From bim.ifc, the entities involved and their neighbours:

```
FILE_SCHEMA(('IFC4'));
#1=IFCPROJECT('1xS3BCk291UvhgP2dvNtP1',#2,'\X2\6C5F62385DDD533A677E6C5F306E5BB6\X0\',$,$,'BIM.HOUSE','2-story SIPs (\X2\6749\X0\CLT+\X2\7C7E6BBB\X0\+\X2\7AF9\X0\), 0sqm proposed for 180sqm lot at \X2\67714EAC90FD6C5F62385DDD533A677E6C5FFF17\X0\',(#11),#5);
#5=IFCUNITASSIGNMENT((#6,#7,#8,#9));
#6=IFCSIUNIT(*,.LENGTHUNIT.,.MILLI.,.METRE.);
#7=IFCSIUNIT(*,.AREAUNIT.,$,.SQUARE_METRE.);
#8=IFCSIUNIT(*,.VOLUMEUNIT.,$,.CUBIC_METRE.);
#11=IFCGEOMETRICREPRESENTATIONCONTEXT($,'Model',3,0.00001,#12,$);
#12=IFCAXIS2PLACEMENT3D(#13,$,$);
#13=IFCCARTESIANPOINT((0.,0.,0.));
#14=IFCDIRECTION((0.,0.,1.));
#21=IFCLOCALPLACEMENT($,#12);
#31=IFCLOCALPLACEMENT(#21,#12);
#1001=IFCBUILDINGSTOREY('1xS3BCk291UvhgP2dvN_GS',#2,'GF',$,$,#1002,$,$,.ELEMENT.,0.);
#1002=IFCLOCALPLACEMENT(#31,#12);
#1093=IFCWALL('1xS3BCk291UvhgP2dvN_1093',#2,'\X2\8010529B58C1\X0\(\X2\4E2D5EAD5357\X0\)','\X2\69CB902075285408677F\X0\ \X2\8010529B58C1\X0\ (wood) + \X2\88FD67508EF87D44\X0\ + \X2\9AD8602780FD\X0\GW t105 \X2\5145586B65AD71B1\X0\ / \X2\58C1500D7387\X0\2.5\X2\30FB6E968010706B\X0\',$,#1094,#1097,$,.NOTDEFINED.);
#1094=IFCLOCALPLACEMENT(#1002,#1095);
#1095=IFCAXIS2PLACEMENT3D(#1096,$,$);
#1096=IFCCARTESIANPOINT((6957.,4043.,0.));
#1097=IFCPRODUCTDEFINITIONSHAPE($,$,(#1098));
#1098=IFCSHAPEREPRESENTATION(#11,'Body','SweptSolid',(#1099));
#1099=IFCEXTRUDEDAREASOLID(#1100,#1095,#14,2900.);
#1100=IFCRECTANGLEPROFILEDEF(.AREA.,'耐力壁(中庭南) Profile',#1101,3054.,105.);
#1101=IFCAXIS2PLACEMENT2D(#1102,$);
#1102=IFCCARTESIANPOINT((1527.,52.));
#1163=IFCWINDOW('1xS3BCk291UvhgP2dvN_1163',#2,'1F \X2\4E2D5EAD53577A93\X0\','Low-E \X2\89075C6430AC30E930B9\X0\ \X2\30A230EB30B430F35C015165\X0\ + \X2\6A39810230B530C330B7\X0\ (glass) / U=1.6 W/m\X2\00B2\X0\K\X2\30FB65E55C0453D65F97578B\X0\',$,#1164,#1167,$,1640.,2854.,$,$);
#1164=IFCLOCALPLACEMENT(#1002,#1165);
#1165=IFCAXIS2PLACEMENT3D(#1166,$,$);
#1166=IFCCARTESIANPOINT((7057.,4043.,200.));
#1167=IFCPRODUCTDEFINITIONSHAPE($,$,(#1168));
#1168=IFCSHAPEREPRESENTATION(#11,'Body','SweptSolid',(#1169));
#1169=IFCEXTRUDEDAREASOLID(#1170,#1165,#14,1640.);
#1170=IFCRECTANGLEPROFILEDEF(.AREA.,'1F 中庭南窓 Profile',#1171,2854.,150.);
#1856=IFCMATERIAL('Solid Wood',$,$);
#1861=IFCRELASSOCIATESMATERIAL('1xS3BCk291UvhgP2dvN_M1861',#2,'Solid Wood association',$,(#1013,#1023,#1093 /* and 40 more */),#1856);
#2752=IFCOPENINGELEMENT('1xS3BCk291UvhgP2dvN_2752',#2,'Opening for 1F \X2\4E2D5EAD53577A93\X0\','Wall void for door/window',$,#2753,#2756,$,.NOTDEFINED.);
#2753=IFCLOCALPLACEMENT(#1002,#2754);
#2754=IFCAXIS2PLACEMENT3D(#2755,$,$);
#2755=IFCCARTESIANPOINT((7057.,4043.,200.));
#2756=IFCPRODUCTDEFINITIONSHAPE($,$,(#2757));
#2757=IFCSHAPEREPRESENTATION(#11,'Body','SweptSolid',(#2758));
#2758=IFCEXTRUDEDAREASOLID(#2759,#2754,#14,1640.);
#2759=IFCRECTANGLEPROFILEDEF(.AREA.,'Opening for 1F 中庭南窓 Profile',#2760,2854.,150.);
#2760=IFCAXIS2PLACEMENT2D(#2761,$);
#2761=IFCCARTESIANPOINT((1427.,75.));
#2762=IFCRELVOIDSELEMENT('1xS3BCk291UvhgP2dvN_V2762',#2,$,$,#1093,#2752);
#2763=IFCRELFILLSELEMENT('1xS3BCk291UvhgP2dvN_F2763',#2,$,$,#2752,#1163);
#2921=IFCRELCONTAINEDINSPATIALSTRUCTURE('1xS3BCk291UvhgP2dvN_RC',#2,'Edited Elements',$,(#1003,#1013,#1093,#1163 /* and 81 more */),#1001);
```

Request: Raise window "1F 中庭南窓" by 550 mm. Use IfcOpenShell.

```python
import numpy as np
import ifcopenshell
import ifcopenshell.api.geometry
import ifcopenshell.util.placement
import ifcopenshell.util.unit

model = ifcopenshell.open("bim.ifc")
unit_scale = ifcopenshell.util.unit.calculate_unit_scale(model)

window = model.by_guid("1xS3BCk291UvhgP2dvN_1163")
opening = window.FillsVoids[0].RelatingOpeningElement
dz = 0.55 / unit_scale

shift = np.array([0.0, 0.0, dz])
# The window is not placed relative to its opening, so move both.
for product in (opening, window):
    matrix = ifcopenshell.util.placement.get_local_placement(product.ObjectPlacement)
    matrix[:3, 3] += shift
    ifcopenshell.api.geometry.edit_object_placement(model, product=product, matrix=matrix, is_si=False)

print(f"moved by {dz * unit_scale:+.3f} m")

model.write("bim_v2.ifc")
```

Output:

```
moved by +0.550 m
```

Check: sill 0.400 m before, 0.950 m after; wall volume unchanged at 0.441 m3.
